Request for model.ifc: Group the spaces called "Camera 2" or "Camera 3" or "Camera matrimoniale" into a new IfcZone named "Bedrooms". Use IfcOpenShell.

First a look at what the model holds.

```python
import ifcopenshell

model = ifcopenshell.open("model.ifc")
print(model.schema)
seen = {}
for space in model.by_type("IfcSpace"):
    seen[space.LongName] = seen.get(space.LongName, 0) + 1
for name, count in sorted(seen.items(), key=str):
    print(count, "x", name)
print("zones:", [z.Name for z in model.by_type("IfcZone")][:20])
```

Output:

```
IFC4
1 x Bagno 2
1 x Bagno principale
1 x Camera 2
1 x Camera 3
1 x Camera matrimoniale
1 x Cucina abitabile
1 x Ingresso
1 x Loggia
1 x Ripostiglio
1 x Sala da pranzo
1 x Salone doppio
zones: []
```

```python
import ifcopenshell
import ifcopenshell.api.group
import ifcopenshell.api.root

model = ifcopenshell.open("model.ifc")

names = {"Camera 2", "Camera 3", "Camera matrimoniale"}
spaces = [s for s in model.by_type("IfcSpace") if s.LongName in names]

zone = ifcopenshell.api.root.create_entity(model, ifc_class="IfcZone", name="Bedrooms")
ifcopenshell.api.group.assign_group(model, products=spaces, group=zone)
print(len(spaces), "spaces in", zone.Name)

model.write("model_v2.ifc")
```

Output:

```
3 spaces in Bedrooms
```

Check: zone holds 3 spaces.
